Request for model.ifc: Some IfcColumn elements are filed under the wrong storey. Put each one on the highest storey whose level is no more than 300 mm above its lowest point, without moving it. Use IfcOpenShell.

First a look at what the model holds.

```python
import ifcopenshell
import ifcopenshell.util.element
import ifcopenshell.util.placement

model = ifcopenshell.open("model.ifc")
print(model.schema)
for storey in model.by_type("IfcBuildingStorey"):
    level = ifcopenshell.util.placement.get_storey_elevation(storey)
    count = sum(e.is_a("IfcColumn") for e in ifcopenshell.util.element.get_contained(storey))
    print(storey.id(), storey.Name, round(level, 3), count, sep=" | ")
```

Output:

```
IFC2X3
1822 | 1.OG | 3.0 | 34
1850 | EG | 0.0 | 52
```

```python
import ifcopenshell
import ifcopenshell.api.spatial
import ifcopenshell.geom
import ifcopenshell.util.element
import ifcopenshell.util.placement
import ifcopenshell.util.shape
import ifcopenshell.util.unit

model = ifcopenshell.open("model.ifc")
unit_scale = ifcopenshell.util.unit.calculate_unit_scale(model)
settings = ifcopenshell.geom.settings()

levels = sorted(
    ((ifcopenshell.util.placement.get_storey_elevation(s) * unit_scale, s) for s in model.by_type("IfcBuildingStorey")),
    key=lambda pair: pair[0],
)

for e in model.by_type("IfcColumn"):
    current = e.ContainedInStructure[0].RelatingStructure if e.ContainedInStructure else None
    if current is None or not current.is_a("IfcBuildingStorey"):
        continue
    shape = ifcopenshell.geom.create_shape(settings, e)
    bottom = ifcopenshell.util.shape.get_shape_bottom_elevation(shape, shape.geometry)
    below = [s for level, s in levels if level <= bottom + 0.3]
    storey = below[-1] if below else levels[0][1]
    if storey != current:
        # assign_container keeps the world position.
        ifcopenshell.api.spatial.assign_container(model, products=[e], relating_structure=storey)
        print(e.id(), current.Name, "->", storey.Name)

model.write("model_rev.ifc")
```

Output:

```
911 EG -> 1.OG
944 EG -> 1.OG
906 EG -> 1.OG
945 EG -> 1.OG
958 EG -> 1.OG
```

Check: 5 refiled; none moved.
